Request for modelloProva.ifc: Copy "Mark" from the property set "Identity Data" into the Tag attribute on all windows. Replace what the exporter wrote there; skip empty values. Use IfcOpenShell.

First a look at what the model holds.

```python
import ifcopenshell
import ifcopenshell.util.element

model = ifcopenshell.open("modelloProva.ifc")
print(model.schema)
windows = model.by_type("IfcWindow")
print(len(windows), "windows")
for e in windows[:8]:
    source = ifcopenshell.util.element.get_pset(e, "Identity Data", "Mark")
    target = e.Tag
    print(e.id(), repr(source), repr(target), sep=" | ")
```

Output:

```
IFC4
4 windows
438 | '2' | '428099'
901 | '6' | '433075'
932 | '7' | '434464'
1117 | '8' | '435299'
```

```python
import ifcopenshell
import ifcopenshell.util.element

model = ifcopenshell.open("modelloProva.ifc")

count = 0
for e in model.by_type("IfcWindow"):
    value = ifcopenshell.util.element.get_pset(e, "Identity Data", "Mark")
    current = e.Tag
    if not value or not value.strip() or current == value:
        continue
    e.Tag = value
    count += 1

print(count, "windows updated")

model.write("modelloProva_rev.ifc")
```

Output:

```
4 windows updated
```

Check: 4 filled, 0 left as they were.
